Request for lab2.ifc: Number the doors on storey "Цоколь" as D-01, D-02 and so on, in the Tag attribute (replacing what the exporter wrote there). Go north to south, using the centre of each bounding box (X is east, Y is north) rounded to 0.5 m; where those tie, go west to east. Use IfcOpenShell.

First a look at what the model holds.

```python
import ifcopenshell
import ifcopenshell.util.element
import ifcopenshell.util.placement

model = ifcopenshell.open("lab2.ifc")
print(model.schema)
storey = next(s for s in model.by_type("IfcBuildingStorey") if s.Name == "Цоколь")
doors = [e for e in ifcopenshell.util.element.get_decomposition(storey) if e.is_a("IfcDoor")]
for e in sorted(doors, key=lambda e: e.id()):
    origin = ifcopenshell.util.placement.get_local_placement(e.ObjectPlacement)[:3, 3]
    print(e.id(), e.Tag, e.Name, origin.round(2) + 0.0, sep=" | ")
```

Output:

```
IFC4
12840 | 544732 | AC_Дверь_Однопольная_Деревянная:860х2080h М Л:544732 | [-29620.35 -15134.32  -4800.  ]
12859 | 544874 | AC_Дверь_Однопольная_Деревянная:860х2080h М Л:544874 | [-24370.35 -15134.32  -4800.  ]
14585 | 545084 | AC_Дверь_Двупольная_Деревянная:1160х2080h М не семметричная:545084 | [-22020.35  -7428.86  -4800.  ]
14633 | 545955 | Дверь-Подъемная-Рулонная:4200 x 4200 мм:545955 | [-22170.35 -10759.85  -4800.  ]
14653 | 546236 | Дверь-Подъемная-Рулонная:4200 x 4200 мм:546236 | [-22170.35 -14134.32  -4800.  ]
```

```python
import ifcopenshell
import ifcopenshell.geom
import ifcopenshell.util.element
import ifcopenshell.util.shape

model = ifcopenshell.open("lab2.ifc")
settings = ifcopenshell.geom.settings()
settings.set("use-world-coords", True)


def centre(element):
    shape = ifcopenshell.geom.create_shape(settings, element)
    return ifcopenshell.util.shape.get_bbox_centroid(shape.geometry)


storey = next(s for s in model.by_type("IfcBuildingStorey") if s.Name == "Цоколь")
doors = [e for e in ifcopenshell.util.element.get_decomposition(storey) if e.is_a("IfcDoor")]

# Insertion points can sit at a corner or the storey origin, so sort by the geometry (in metres).
centres = {e: centre(e) for e in doors}
doors.sort(key=lambda e: (-round(centres[e][1] / 0.5), centres[e][0]))

for i, e in enumerate(doors, start=1):
    number = f"D-{i:02d}"
    e.Tag = number
    print(e.id(), number)

model.write("lab2_updated.ifc")
```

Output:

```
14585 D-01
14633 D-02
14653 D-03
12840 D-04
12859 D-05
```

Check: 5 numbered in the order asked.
